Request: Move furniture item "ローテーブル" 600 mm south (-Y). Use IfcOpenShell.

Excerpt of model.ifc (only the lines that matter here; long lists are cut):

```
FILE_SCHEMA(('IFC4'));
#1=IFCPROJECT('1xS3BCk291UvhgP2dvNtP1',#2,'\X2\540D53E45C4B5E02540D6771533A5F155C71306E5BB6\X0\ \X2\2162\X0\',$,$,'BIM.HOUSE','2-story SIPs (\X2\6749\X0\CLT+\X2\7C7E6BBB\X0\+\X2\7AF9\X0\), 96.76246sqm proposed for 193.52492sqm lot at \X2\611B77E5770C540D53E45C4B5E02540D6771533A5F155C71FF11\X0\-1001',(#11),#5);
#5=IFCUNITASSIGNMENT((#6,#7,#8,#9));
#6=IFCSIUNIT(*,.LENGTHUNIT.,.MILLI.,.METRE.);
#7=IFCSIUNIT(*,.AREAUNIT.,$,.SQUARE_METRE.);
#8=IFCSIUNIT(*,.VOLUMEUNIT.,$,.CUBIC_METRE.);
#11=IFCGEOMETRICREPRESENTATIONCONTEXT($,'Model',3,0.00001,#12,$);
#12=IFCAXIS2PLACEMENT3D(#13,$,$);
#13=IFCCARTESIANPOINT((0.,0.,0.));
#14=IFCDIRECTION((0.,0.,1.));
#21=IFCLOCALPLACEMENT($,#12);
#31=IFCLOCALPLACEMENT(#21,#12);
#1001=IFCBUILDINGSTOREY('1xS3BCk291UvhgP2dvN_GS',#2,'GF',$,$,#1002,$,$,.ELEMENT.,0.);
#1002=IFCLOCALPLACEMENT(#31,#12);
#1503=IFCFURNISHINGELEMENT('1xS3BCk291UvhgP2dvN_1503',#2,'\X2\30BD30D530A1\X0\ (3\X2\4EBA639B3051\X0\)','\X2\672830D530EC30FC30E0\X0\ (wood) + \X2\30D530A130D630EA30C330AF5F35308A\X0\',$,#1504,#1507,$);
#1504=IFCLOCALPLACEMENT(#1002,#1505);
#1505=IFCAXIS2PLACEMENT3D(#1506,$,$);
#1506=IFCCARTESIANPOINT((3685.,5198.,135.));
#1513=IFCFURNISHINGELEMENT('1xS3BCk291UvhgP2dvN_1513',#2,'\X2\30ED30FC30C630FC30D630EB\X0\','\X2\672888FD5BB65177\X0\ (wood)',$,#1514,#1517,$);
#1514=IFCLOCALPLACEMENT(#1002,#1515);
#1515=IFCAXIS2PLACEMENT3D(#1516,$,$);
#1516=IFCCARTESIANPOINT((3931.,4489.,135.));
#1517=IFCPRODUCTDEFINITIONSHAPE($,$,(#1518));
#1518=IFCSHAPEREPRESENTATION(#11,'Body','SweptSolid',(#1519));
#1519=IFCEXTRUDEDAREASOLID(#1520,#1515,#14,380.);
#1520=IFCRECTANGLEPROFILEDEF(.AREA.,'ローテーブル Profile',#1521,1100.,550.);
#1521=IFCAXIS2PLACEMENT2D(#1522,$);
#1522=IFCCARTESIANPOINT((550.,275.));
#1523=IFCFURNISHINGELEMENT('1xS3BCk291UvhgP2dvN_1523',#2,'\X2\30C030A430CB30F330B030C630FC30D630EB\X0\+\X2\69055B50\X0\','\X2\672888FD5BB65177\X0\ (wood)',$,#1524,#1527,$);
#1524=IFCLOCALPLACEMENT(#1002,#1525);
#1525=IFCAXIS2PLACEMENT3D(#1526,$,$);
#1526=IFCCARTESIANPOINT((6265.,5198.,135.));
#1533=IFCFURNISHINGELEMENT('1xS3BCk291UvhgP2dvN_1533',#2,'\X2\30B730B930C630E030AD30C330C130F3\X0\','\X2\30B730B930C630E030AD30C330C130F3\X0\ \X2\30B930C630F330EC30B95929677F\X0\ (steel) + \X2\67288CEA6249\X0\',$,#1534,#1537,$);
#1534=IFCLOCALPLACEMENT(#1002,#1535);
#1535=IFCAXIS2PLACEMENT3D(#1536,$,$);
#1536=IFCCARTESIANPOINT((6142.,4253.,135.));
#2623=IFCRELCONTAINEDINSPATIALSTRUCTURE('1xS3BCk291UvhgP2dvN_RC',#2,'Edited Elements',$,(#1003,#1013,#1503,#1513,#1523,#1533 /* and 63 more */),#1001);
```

```python
import ifcopenshell
import ifcopenshell.api.geometry
import ifcopenshell.util.placement

model = ifcopenshell.open("model.ifc")

item = model.by_guid("1xS3BCk291UvhgP2dvN_1513")
matrix = ifcopenshell.util.placement.get_local_placement(item.ObjectPlacement)
matrix[1, 3] -= 600.0
ifcopenshell.api.geometry.edit_object_placement(model, product=item, matrix=matrix, is_si=False)

print(ifcopenshell.util.placement.get_local_placement(item.ObjectPlacement).round(3) + 0.0)

model.write("model_updated.ifc")
```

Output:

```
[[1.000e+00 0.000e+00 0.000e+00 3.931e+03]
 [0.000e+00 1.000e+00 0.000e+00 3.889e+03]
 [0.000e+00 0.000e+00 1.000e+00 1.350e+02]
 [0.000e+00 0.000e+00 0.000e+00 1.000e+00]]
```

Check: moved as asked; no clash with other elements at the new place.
